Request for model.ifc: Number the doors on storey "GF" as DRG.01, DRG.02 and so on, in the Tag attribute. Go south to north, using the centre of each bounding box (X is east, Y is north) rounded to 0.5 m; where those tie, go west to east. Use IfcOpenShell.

First a look at what the model holds.

```python
import ifcopenshell
import ifcopenshell.util.element
import ifcopenshell.util.placement

model = ifcopenshell.open("model.ifc")
print(model.schema)
storey = next(s for s in model.by_type("IfcBuildingStorey") if s.Name == "GF")
doors = [e for e in ifcopenshell.util.element.get_decomposition(storey) if e.is_a("IfcDoor")]
for e in sorted(doors, key=lambda e: e.id()):
    origin = ifcopenshell.util.placement.get_local_placement(e.ObjectPlacement)[:3, 3]
    print(e.id(), e.Tag, e.Name, origin.round(2) + 0.0, sep=" | ")
```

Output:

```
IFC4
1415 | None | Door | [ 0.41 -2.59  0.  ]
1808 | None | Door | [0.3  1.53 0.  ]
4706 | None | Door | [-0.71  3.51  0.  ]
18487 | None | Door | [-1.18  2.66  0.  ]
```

```python
import ifcopenshell
import ifcopenshell.geom
import ifcopenshell.util.element
import ifcopenshell.util.shape

model = ifcopenshell.open("model.ifc")
settings = ifcopenshell.geom.settings()
settings.set("use-world-coords", True)


def centre(element):
    shape = ifcopenshell.geom.create_shape(settings, element)
    return ifcopenshell.util.shape.get_bbox_centroid(shape.geometry)


storey = next(s for s in model.by_type("IfcBuildingStorey") if s.Name == "GF")
doors = [e for e in ifcopenshell.util.element.get_decomposition(storey) if e.is_a("IfcDoor")]

# Insertion points can sit at a corner or the storey origin, so sort by the geometry (in metres).
centres = {e: centre(e) for e in doors}
doors.sort(key=lambda e: (round(centres[e][1] / 0.5), centres[e][0]))

for i, e in enumerate(doors, start=1):
    number = f"DRG.{i:02d}"
    e.Tag = number
    print(e.id(), number)

model.write("model-out.ifc")
```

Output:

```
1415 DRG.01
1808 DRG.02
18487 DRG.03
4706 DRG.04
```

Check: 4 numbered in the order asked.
